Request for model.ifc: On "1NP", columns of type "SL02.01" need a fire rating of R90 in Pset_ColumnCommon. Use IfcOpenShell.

First a look at what the model holds.

```python
import ifcopenshell
import ifcopenshell.util.element

model = ifcopenshell.open("model.ifc")
print(model.schema)
storey = next(s for s in model.by_type("IfcBuildingStorey") if s.Name == "1NP")
columns = [e for e in ifcopenshell.util.element.get_decomposition(storey) if e.is_a("IfcColumn")]
seen = {}
for e in columns:
    element_type = ifcopenshell.util.element.get_type(e)
    key = (element_type.Name if element_type != e and element_type else None, ifcopenshell.util.element.get_pset(e, "Pset_ColumnCommon", "FireRating"))
    seen[key] = seen.get(key, 0) + 1
for (name, value), count in sorted(seen.items(), key=str):
    print(count, "x", name, "|", value)
```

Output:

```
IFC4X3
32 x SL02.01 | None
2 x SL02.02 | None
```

```python
import ifcopenshell
import ifcopenshell.api.pset
import ifcopenshell.util.element

model = ifcopenshell.open("model.ifc")

storey = next(s for s in model.by_type("IfcBuildingStorey") if s.Name == "1NP")
columns = [e for e in ifcopenshell.util.element.get_decomposition(storey) if e.is_a("IfcColumn")]

count = 0
for e in columns:
    element_type = ifcopenshell.util.element.get_type(e)
    if element_type in (None, e) or element_type.Name != "SL02.01":
        continue
    # add_pset returns the element's existing set when there is one.
    pset = ifcopenshell.api.pset.add_pset(model, product=e, name="Pset_ColumnCommon")
    ifcopenshell.api.pset.edit_pset(model, pset=pset, properties={"FireRating": "R90"})
    count += 1

print(count, "columns updated")

model.write("model-out.ifc")
```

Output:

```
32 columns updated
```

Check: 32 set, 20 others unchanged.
